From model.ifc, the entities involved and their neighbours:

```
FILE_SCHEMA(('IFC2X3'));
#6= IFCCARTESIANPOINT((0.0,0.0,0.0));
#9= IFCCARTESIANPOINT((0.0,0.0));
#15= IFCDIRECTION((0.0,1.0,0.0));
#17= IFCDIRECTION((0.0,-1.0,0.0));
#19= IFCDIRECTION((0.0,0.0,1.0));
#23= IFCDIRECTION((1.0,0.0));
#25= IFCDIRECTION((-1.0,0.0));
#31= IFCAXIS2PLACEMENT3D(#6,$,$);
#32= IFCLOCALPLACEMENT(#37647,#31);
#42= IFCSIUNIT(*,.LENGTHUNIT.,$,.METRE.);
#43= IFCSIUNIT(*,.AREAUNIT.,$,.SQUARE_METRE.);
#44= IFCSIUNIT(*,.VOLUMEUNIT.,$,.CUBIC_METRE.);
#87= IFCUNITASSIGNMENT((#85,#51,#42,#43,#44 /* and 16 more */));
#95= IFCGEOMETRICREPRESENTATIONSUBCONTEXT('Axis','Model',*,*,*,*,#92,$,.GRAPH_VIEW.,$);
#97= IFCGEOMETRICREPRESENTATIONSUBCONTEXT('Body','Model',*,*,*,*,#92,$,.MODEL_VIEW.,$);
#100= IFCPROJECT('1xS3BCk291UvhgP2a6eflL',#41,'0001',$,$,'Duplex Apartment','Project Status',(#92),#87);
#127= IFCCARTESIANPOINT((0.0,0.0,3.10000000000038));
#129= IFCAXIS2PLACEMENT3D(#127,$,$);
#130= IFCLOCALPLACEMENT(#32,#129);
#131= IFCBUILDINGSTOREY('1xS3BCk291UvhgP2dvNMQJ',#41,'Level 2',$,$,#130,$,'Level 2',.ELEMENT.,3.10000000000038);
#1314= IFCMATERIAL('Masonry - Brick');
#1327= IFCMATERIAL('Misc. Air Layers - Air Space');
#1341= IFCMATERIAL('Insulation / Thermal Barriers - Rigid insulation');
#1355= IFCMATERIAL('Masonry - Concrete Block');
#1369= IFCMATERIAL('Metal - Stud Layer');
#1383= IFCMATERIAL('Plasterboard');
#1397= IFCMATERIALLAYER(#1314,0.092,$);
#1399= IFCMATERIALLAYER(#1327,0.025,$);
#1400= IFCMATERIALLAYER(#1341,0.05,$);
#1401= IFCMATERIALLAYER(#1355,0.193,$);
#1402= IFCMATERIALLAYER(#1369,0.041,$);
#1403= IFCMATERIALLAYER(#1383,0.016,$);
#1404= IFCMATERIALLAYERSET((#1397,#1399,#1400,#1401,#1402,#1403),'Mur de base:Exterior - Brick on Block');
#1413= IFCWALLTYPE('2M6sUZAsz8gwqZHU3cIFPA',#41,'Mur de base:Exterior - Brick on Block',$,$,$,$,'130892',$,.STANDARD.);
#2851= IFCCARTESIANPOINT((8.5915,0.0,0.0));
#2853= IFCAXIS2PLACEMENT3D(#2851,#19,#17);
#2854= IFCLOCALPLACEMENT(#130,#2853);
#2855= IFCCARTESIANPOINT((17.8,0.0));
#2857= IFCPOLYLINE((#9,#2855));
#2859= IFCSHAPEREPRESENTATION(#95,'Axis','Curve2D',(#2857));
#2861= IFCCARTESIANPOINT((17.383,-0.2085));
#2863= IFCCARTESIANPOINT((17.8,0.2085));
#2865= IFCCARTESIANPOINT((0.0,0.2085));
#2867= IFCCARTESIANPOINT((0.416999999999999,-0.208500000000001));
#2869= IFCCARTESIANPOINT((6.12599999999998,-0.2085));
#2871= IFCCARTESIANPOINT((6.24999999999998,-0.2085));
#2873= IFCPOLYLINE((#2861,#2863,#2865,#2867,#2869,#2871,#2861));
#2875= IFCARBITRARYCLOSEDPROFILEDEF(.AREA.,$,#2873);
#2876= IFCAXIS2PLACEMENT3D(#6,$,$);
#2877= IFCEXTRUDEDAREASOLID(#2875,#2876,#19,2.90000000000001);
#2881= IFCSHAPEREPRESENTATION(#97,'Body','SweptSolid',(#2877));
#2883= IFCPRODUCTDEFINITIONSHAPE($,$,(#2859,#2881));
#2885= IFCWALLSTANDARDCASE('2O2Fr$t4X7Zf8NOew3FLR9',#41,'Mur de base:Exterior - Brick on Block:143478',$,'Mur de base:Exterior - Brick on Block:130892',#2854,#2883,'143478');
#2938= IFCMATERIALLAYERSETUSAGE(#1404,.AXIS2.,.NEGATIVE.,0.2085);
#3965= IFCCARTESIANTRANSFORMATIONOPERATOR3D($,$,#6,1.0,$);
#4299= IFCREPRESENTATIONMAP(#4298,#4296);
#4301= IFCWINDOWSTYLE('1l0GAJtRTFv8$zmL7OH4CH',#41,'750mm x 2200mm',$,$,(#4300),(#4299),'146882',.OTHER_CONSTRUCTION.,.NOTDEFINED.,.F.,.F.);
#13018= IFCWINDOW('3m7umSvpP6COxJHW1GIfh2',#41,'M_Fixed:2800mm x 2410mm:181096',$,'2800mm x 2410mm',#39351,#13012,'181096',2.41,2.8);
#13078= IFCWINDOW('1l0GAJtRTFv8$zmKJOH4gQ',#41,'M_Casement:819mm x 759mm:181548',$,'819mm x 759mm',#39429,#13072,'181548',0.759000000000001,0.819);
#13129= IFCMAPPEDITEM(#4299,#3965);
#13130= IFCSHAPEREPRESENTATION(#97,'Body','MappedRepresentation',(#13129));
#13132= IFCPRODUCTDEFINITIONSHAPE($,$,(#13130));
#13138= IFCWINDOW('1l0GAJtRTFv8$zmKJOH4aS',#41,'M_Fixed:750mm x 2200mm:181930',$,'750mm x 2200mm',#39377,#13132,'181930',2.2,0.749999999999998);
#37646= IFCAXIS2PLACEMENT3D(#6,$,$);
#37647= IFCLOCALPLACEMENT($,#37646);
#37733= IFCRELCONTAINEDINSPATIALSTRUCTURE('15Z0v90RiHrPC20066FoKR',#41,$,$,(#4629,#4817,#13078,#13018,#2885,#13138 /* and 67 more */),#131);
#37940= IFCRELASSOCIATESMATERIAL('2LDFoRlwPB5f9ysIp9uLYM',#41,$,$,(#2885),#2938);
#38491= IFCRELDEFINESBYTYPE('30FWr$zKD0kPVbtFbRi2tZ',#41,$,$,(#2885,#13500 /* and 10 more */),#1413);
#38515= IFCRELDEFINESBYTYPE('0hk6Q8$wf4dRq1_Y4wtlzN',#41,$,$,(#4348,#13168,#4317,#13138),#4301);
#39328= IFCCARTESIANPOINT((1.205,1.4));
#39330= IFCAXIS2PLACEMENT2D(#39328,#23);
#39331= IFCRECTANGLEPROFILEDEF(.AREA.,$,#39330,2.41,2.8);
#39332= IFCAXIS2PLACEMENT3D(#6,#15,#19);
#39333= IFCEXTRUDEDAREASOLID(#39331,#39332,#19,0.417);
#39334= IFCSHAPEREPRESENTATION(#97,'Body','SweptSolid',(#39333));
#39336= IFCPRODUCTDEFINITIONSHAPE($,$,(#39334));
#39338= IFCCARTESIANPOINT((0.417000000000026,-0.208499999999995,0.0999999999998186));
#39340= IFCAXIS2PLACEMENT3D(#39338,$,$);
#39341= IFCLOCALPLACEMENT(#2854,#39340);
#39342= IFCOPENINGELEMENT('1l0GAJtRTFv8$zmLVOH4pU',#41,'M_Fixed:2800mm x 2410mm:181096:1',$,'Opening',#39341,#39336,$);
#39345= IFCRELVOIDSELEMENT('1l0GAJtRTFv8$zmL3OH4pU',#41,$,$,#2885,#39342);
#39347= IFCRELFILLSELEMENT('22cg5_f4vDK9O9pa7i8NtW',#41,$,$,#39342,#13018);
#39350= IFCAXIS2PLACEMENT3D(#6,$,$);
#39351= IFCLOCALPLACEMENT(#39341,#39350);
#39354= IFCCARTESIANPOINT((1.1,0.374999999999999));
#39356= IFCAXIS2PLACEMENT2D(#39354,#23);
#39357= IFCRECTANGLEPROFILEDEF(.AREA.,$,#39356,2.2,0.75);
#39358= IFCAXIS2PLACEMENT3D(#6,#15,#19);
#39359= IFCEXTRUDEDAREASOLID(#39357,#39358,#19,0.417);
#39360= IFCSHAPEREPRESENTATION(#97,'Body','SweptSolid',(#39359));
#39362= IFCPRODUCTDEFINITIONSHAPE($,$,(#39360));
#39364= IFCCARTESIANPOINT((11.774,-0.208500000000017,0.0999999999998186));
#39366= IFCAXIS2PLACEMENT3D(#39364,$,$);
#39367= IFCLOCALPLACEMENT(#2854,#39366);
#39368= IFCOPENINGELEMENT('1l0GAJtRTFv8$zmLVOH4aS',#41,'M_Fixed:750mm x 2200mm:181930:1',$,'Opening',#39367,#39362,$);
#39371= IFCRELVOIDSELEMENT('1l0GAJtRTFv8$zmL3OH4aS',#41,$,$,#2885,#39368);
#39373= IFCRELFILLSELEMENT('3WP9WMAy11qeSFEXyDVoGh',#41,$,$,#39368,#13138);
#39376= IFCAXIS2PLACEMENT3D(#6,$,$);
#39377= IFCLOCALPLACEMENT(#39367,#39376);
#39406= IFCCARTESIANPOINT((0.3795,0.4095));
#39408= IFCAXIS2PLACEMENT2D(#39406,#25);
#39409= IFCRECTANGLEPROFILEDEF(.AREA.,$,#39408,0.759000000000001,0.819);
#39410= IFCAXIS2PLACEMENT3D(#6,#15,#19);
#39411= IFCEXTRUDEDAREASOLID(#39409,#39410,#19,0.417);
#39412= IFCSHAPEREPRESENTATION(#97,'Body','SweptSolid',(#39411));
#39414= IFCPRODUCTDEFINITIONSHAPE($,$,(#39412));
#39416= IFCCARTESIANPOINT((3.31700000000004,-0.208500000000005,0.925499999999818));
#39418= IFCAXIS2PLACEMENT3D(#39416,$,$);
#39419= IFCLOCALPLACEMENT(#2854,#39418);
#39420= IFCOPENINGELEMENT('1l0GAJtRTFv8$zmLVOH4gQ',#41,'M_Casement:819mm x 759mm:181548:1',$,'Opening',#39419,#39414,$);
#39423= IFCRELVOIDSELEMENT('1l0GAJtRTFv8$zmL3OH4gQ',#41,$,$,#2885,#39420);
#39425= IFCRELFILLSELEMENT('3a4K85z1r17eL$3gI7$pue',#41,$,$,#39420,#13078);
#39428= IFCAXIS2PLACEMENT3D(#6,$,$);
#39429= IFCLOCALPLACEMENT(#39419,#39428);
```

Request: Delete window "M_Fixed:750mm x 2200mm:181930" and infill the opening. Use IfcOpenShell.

```python
import ifcopenshell
import ifcopenshell.api.feature
import ifcopenshell.api.root
import ifcopenshell.geom
import ifcopenshell.util.shape

model = ifcopenshell.open("model.ifc")
settings = ifcopenshell.geom.settings()


def volume(element):
    """Net volume in cubic metres, openings subtracted."""
    shape = ifcopenshell.geom.create_shape(settings, element)
    return ifcopenshell.util.shape.get_volume(shape.geometry)


window = model.by_guid("1l0GAJtRTFv8$zmKJOH4aS")
opening = window.FillsVoids[0].RelatingOpeningElement
wall = opening.VoidsElements[0].RelatingBuildingElement
before = volume(wall)

ifcopenshell.api.root.remove_product(model, product=window)
ifcopenshell.api.feature.remove_feature(model, feature=opening)

after = volume(wall)

print(f"wall volume {before:.3f} -> {after:.3f} m3")

model.write("model_rev.ifc")
```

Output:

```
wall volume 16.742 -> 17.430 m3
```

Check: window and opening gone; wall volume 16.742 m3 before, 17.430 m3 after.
